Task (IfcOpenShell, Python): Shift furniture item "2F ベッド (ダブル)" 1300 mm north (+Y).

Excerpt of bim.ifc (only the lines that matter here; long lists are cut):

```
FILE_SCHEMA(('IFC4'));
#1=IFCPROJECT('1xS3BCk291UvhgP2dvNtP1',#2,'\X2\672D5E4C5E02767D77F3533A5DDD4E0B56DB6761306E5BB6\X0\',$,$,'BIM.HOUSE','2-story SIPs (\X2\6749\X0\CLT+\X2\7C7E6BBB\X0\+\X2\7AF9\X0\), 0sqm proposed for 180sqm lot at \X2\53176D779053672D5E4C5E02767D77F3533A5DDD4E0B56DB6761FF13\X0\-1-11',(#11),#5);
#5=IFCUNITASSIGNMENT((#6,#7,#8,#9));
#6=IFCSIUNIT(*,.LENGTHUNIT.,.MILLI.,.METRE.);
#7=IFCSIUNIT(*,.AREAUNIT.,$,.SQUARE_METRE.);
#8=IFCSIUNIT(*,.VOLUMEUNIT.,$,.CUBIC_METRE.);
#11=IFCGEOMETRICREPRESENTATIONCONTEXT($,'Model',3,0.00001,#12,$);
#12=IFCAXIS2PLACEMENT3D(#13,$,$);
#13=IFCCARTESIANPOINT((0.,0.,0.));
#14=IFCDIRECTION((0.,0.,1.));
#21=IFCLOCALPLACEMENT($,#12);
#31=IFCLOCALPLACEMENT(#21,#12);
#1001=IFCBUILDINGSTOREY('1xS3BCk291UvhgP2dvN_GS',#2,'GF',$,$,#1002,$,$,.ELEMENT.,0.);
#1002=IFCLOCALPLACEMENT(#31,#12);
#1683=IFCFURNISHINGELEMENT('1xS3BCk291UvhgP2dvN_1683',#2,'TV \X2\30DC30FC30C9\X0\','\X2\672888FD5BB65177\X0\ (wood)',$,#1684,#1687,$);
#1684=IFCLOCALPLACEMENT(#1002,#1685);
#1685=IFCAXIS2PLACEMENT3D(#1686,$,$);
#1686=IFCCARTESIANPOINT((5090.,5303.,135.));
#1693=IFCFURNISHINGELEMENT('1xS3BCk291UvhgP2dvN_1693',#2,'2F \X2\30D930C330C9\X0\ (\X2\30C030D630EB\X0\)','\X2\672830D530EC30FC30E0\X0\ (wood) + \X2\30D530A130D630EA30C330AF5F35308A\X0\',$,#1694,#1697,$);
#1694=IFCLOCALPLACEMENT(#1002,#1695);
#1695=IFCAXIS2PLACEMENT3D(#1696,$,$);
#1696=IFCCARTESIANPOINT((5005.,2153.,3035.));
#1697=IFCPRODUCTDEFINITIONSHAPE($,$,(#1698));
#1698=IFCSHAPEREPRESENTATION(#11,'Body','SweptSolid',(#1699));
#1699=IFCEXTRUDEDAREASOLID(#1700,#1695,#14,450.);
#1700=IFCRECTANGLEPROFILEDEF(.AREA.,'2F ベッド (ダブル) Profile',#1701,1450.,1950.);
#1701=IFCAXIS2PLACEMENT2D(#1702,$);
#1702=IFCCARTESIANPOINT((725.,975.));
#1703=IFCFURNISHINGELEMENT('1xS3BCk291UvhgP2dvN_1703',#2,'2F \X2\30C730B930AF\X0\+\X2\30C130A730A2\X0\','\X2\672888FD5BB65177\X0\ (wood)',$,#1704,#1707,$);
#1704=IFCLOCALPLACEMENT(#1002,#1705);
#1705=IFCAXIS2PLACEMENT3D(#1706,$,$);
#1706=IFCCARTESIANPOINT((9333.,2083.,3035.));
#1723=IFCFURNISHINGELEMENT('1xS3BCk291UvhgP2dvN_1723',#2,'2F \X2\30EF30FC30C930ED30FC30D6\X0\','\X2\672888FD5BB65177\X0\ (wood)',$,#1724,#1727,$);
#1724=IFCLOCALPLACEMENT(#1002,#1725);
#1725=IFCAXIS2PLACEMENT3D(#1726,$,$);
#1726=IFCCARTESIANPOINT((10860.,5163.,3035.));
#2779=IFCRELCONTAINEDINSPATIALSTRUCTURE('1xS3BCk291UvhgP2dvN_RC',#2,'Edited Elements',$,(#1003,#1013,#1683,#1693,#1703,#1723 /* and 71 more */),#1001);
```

```python
import ifcopenshell
import ifcopenshell.api.geometry
import ifcopenshell.util.placement

model = ifcopenshell.open("bim.ifc")

item = model.by_guid("1xS3BCk291UvhgP2dvN_1693")
matrix = ifcopenshell.util.placement.get_local_placement(item.ObjectPlacement)
matrix[1, 3] += 1300.0
ifcopenshell.api.geometry.edit_object_placement(model, product=item, matrix=matrix, is_si=False)

print(ifcopenshell.util.placement.get_local_placement(item.ObjectPlacement).round(3) + 0.0)

model.write("bim_rev.ifc")
```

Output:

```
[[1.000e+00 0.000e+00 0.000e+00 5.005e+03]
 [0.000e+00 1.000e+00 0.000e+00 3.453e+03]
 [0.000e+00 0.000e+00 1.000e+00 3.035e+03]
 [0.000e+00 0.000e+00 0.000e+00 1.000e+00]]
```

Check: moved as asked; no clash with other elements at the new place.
